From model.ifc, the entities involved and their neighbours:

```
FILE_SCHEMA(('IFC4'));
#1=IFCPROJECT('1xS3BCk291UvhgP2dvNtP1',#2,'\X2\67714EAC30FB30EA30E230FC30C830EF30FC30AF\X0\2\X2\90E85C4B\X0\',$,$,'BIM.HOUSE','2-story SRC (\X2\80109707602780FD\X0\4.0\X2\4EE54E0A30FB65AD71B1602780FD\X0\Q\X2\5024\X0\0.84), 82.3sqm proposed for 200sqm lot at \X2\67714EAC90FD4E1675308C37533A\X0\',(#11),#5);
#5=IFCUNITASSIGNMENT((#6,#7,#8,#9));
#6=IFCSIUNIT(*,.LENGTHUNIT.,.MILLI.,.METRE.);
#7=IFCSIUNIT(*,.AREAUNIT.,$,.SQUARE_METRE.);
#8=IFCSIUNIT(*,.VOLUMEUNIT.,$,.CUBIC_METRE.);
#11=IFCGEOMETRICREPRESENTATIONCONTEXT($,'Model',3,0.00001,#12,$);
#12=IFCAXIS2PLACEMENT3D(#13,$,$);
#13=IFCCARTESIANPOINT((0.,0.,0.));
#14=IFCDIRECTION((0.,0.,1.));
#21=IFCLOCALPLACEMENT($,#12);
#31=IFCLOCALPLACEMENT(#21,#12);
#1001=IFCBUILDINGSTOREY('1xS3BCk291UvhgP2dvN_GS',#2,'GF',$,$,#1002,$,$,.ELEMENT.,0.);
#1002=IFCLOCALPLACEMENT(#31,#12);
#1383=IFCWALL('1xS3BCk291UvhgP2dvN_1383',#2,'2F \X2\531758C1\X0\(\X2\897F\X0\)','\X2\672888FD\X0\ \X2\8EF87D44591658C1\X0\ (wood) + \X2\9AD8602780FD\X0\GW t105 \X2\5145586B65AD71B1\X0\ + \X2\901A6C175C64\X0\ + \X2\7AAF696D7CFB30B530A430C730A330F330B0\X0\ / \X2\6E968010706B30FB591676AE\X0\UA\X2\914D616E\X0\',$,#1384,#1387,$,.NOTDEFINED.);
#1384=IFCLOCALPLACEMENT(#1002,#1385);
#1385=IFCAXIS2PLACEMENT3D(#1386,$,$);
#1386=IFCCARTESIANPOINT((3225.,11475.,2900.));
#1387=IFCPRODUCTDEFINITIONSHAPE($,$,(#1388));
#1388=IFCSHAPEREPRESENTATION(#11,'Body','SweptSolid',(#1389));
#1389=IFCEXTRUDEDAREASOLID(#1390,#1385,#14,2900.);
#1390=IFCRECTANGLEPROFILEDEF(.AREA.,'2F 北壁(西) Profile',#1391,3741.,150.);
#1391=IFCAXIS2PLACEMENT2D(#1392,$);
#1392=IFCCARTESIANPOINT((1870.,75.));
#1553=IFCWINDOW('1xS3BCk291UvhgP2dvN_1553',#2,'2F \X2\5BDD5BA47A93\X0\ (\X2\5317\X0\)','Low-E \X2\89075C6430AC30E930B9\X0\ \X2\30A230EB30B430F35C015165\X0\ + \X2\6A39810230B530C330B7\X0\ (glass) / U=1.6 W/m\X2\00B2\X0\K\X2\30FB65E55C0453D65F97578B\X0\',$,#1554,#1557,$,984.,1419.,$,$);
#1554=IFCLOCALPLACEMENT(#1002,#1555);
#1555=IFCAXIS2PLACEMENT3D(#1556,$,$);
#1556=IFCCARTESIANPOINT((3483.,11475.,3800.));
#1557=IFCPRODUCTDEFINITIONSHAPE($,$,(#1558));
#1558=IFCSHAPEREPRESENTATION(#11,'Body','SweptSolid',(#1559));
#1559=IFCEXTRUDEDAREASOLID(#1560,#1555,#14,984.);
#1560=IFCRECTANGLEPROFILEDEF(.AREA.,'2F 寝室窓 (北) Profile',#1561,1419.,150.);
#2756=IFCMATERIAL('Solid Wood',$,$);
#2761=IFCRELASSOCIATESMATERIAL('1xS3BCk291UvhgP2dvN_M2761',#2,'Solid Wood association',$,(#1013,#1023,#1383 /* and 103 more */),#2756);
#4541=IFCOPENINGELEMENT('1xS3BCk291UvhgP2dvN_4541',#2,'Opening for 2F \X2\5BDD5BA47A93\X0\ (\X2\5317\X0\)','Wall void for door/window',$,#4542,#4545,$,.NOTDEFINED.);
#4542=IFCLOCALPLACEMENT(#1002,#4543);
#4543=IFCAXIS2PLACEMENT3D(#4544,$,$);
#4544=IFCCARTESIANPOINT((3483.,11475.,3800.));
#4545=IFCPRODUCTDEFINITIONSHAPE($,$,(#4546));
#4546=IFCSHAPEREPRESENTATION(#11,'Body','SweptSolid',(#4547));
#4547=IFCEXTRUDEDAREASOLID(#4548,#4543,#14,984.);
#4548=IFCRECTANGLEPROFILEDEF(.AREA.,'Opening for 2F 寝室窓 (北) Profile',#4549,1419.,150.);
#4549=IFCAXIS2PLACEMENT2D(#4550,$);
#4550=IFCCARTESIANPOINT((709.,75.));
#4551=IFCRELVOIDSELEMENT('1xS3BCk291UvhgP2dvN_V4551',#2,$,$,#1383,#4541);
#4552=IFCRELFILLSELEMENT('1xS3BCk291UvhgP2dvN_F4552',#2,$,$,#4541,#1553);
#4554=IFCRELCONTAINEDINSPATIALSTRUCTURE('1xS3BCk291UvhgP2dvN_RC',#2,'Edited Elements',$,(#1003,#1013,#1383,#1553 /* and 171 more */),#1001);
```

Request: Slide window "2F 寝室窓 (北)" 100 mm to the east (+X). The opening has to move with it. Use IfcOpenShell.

```python
import ifcopenshell
import ifcopenshell.api.geometry
import ifcopenshell.util.placement
import ifcopenshell.util.unit

model = ifcopenshell.open("model.ifc")
unit_scale = ifcopenshell.util.unit.calculate_unit_scale(model)

window = model.by_guid("1xS3BCk291UvhgP2dvN_1553")
opening = window.FillsVoids[0].RelatingOpeningElement
wall = opening.VoidsElements[0].RelatingBuildingElement

wall_matrix = ifcopenshell.util.placement.get_local_placement(wall.ObjectPlacement)
shift = wall_matrix[:3, 0] * 0.1 / unit_scale
before = ifcopenshell.util.placement.get_local_placement(window.ObjectPlacement)[:3, 3].copy()

# The window is not placed relative to its opening, so move both.
for product in (opening, window):
    matrix = ifcopenshell.util.placement.get_local_placement(product.ObjectPlacement)
    matrix[:3, 3] += shift
    ifcopenshell.api.geometry.edit_object_placement(model, product=product, matrix=matrix, is_si=False)

after = ifcopenshell.util.placement.get_local_placement(window.ObjectPlacement)[:3, 3]
print("window moved by", (after - before).round(3) + 0.0)

model.write("model_edited.ifc")
```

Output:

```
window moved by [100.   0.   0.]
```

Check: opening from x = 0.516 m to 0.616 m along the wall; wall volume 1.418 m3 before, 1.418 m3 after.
